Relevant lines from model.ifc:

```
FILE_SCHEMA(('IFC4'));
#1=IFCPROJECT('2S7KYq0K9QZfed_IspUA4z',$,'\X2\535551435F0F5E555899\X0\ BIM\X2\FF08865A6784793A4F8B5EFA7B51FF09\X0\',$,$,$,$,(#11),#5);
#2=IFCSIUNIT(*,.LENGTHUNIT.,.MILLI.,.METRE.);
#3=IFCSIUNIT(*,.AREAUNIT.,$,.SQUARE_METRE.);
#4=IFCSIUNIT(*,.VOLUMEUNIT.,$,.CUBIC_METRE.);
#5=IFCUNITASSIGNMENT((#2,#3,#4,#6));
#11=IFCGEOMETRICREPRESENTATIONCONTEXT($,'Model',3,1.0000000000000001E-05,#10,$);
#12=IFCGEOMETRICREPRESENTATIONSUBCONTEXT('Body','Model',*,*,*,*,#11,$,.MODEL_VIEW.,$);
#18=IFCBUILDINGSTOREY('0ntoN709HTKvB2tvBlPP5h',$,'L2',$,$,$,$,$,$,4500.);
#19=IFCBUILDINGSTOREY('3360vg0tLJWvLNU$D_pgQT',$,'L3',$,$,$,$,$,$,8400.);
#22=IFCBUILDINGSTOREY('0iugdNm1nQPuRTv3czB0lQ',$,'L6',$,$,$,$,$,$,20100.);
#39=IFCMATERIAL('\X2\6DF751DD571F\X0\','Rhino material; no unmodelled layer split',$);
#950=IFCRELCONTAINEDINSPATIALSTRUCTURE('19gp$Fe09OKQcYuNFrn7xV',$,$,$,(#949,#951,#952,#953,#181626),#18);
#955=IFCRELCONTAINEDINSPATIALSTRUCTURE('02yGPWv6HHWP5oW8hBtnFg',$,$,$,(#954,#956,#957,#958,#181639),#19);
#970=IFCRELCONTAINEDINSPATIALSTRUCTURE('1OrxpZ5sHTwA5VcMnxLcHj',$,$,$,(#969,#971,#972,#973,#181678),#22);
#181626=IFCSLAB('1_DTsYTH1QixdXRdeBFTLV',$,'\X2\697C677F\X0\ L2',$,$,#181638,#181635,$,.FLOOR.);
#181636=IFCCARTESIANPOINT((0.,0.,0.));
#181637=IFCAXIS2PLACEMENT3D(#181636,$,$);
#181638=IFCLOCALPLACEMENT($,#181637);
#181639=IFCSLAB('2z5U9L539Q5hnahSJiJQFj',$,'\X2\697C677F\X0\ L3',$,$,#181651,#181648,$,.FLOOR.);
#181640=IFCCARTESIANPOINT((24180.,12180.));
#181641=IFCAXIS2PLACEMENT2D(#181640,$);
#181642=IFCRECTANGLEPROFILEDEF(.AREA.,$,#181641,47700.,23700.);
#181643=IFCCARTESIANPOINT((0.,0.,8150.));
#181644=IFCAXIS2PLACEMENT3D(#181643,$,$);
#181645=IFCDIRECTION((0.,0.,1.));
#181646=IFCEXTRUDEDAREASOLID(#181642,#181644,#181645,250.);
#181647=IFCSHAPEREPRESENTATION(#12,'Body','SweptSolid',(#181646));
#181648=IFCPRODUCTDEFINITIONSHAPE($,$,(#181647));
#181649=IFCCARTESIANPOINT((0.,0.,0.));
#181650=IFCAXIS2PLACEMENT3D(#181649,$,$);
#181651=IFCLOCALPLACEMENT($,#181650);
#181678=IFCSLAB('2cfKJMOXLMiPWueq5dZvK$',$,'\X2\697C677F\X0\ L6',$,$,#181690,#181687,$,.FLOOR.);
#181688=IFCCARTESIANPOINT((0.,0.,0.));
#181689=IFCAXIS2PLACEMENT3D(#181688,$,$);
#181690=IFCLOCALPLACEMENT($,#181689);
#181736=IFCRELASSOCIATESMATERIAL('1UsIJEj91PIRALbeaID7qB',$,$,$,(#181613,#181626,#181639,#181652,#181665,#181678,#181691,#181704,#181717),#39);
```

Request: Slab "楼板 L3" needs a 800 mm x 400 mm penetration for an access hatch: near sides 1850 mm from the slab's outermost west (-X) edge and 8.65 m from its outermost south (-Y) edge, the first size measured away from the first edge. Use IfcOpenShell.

```python
import numpy as np
import ifcopenshell
import ifcopenshell.api.feature
import ifcopenshell.api.geometry
import ifcopenshell.api.root
import ifcopenshell.geom
import ifcopenshell.util.placement
import ifcopenshell.util.representation
import ifcopenshell.util.shape
import ifcopenshell.util.unit

model = ifcopenshell.open("model.ifc")
unit_scale = ifcopenshell.util.unit.calculate_unit_scale(model)
settings = ifcopenshell.geom.settings()


def volume(element):
    """Net volume in cubic metres, openings subtracted."""
    shape = ifcopenshell.geom.create_shape(settings, element)
    return ifcopenshell.util.shape.get_volume(shape.geometry)


slab = model.by_guid("2z5U9L539Q5hnahSJiJQFj")
before = volume(slab)

# Extent in the slab's own axes, in metres. The edges named are its -X and -Y sides.
slab_shape = ifcopenshell.geom.create_shape(settings, slab)
vertices = ifcopenshell.util.shape.get_vertices(slab_shape.geometry)
x_min, y_min, bottom = vertices.min(axis=0)
top = vertices[:, 2].max()

opening = ifcopenshell.api.root.create_entity(model, ifc_class="IfcOpeningElement", name="Access hatch opening", predefined_type="OPENING")
context = ifcopenshell.util.representation.get_context(model, "Model", "Body", "MODEL_VIEW")
width, depth = 0.8, 0.4
outline = [(0.0, 0.0), (width, 0.0), (width, depth), (0.0, depth), (0.0, 0.0)]
# Overshoot both faces by 50 mm so the cut is clean.
shape = ifcopenshell.api.geometry.add_slab_representation(
    model, context=context, depth=top - bottom + 0.1, polyline=outline
)
ifcopenshell.api.geometry.assign_representation(model, product=opening, representation=shape)

matrix = ifcopenshell.util.placement.get_local_placement(slab.ObjectPlacement)
matrix[:, 3] = matrix @ np.append(np.array([x_min + 1.85, y_min + 8.65, bottom - 0.05]) / unit_scale, 1.0)
ifcopenshell.api.geometry.edit_object_placement(model, product=opening, matrix=matrix, is_si=False)
ifcopenshell.api.feature.add_feature(model, feature=opening, element=slab)

after = volume(slab)

print(f"slab volume {before:.3f} -> {after:.3f} m3")

model.write("model_v2.ifc")
```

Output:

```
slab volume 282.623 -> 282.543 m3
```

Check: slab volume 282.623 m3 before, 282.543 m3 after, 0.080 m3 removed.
